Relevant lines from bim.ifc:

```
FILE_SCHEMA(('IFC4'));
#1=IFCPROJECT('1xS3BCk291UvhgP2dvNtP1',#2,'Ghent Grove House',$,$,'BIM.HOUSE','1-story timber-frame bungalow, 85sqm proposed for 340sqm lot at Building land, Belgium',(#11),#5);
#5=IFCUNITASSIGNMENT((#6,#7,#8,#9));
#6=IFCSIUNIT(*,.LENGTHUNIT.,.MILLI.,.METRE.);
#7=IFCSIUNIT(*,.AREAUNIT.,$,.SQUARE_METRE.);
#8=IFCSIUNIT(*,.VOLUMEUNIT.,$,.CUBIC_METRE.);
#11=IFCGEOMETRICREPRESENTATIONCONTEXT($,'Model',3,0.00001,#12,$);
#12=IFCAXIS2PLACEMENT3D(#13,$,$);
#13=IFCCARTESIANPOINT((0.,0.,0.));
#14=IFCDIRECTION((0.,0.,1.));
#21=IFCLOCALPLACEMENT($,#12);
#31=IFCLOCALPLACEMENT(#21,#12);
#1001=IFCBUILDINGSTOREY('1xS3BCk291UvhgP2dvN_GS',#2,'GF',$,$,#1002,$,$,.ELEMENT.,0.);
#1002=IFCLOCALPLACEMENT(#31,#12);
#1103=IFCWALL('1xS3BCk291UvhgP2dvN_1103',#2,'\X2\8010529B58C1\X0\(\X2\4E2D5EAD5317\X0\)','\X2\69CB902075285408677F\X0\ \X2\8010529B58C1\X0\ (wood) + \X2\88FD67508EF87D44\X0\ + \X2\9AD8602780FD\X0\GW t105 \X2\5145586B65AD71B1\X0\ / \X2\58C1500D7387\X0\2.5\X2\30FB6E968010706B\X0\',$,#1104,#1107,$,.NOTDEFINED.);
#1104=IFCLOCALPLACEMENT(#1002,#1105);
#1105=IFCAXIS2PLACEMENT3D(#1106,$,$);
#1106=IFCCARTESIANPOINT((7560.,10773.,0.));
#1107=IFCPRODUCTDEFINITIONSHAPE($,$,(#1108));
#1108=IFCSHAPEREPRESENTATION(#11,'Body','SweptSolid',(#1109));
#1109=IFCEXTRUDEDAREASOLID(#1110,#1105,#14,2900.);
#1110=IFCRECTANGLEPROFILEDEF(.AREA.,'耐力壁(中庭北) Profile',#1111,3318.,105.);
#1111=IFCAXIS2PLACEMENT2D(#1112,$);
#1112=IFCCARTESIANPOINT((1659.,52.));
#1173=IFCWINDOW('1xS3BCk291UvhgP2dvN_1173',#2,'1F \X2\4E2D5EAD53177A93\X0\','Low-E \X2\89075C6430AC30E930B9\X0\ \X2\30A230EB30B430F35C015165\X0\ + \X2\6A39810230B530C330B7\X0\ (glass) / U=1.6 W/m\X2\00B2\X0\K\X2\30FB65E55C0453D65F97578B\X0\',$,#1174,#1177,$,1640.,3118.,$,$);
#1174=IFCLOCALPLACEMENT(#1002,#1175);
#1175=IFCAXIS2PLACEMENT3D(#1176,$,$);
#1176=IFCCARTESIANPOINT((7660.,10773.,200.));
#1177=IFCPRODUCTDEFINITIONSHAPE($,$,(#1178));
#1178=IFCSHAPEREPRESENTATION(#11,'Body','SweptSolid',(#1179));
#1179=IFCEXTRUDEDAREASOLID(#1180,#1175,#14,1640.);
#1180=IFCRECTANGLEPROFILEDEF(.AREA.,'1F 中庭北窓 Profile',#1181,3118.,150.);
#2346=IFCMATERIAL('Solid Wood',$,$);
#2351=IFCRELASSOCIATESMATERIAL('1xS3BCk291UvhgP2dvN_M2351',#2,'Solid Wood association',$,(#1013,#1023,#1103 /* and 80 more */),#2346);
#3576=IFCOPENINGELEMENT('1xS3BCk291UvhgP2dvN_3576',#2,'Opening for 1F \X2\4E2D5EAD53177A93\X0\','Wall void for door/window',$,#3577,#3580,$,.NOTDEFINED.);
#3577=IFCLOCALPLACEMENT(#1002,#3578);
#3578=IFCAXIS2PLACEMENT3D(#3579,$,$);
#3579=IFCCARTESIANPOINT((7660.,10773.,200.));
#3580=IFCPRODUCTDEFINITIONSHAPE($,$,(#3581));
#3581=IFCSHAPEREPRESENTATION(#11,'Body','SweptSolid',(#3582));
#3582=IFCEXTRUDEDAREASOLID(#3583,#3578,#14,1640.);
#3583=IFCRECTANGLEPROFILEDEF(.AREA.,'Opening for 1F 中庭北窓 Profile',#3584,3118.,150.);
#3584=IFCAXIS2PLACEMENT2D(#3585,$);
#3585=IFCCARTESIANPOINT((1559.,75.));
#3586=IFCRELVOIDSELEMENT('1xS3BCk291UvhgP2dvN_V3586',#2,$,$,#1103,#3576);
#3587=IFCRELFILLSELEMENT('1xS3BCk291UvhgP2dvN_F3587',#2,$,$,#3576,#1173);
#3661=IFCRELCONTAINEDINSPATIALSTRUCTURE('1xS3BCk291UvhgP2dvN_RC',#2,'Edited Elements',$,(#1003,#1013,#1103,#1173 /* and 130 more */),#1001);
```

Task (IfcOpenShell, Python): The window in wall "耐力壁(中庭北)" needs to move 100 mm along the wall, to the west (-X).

```python
import ifcopenshell
import ifcopenshell.api.geometry
import ifcopenshell.util.placement

model = ifcopenshell.open("bim.ifc")

window = model.by_guid("1xS3BCk291UvhgP2dvN_1173")
opening = window.FillsVoids[0].RelatingOpeningElement
wall = opening.VoidsElements[0].RelatingBuildingElement

wall_matrix = ifcopenshell.util.placement.get_local_placement(wall.ObjectPlacement)
shift = wall_matrix[:3, 0] * -100.0
before = ifcopenshell.util.placement.get_local_placement(window.ObjectPlacement)[:3, 3].copy()

# The window is not placed relative to its opening, so move both.
for product in (opening, window):
    matrix = ifcopenshell.util.placement.get_local_placement(product.ObjectPlacement)
    matrix[:3, 3] += shift
    ifcopenshell.api.geometry.edit_object_placement(model, product=product, matrix=matrix, is_si=False)

after = ifcopenshell.util.placement.get_local_placement(window.ObjectPlacement)[:3, 3]
print("window moved by", (after - before).round(3) + 0.0)

model.write("bim_edited.ifc")
```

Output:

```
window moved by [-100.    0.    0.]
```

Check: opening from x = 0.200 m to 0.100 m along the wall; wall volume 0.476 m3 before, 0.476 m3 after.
